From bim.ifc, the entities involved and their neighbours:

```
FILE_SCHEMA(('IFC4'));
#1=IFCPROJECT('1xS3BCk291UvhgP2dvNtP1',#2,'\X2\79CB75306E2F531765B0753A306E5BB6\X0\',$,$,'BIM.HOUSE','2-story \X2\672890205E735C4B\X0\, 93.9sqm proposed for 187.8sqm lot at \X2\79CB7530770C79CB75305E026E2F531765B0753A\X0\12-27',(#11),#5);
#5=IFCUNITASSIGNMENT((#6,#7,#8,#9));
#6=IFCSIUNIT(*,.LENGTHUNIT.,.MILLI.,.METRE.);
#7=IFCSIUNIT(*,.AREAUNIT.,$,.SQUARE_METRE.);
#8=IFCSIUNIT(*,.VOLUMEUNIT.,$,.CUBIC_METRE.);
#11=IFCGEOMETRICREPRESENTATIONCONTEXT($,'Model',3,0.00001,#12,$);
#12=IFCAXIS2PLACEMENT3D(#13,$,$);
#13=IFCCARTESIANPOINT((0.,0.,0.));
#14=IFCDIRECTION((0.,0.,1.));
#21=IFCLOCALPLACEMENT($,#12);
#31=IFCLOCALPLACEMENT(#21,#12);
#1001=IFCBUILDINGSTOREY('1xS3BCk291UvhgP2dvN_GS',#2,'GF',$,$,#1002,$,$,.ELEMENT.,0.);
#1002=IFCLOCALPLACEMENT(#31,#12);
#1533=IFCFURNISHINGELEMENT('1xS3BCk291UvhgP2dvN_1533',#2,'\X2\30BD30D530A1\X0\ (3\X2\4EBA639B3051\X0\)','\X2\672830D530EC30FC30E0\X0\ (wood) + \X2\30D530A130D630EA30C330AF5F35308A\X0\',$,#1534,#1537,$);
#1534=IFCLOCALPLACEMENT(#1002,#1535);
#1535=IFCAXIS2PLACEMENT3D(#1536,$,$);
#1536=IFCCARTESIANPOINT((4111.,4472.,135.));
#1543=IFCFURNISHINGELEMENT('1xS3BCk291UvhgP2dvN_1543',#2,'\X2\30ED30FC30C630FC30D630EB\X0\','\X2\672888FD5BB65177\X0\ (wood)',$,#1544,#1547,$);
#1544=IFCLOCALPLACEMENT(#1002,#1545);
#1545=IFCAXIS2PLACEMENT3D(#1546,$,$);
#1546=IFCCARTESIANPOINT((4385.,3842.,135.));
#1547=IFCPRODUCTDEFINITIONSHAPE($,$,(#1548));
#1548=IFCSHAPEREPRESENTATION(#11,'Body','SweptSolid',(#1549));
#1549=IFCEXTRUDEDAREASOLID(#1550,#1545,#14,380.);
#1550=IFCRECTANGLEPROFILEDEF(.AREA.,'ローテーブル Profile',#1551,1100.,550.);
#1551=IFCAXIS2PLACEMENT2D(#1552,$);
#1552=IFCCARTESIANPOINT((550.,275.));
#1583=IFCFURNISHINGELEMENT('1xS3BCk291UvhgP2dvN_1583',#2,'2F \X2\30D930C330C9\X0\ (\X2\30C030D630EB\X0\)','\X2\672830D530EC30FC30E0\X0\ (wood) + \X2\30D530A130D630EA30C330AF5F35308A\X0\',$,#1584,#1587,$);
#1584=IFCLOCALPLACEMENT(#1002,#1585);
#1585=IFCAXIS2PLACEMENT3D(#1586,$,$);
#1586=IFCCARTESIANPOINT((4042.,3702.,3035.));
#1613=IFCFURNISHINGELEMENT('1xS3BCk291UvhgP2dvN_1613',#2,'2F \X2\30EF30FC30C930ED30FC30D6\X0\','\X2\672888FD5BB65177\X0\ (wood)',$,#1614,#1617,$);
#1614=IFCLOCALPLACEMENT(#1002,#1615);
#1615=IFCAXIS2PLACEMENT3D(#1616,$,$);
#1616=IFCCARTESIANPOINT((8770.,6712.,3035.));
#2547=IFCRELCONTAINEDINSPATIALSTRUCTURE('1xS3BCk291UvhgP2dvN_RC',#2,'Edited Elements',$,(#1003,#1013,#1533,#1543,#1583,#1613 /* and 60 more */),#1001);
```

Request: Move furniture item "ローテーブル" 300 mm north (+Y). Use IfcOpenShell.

```python
import ifcopenshell
import ifcopenshell.api.geometry
import ifcopenshell.util.placement

model = ifcopenshell.open("bim.ifc")

item = model.by_guid("1xS3BCk291UvhgP2dvN_1543")
matrix = ifcopenshell.util.placement.get_local_placement(item.ObjectPlacement)
matrix[1, 3] += 300.0
ifcopenshell.api.geometry.edit_object_placement(model, product=item, matrix=matrix, is_si=False)

print(ifcopenshell.util.placement.get_local_placement(item.ObjectPlacement).round(3) + 0.0)

model.write("bim_updated.ifc")
```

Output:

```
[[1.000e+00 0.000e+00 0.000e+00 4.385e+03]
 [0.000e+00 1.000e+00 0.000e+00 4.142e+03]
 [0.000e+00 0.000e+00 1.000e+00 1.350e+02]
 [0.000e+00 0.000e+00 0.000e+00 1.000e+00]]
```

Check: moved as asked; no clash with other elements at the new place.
